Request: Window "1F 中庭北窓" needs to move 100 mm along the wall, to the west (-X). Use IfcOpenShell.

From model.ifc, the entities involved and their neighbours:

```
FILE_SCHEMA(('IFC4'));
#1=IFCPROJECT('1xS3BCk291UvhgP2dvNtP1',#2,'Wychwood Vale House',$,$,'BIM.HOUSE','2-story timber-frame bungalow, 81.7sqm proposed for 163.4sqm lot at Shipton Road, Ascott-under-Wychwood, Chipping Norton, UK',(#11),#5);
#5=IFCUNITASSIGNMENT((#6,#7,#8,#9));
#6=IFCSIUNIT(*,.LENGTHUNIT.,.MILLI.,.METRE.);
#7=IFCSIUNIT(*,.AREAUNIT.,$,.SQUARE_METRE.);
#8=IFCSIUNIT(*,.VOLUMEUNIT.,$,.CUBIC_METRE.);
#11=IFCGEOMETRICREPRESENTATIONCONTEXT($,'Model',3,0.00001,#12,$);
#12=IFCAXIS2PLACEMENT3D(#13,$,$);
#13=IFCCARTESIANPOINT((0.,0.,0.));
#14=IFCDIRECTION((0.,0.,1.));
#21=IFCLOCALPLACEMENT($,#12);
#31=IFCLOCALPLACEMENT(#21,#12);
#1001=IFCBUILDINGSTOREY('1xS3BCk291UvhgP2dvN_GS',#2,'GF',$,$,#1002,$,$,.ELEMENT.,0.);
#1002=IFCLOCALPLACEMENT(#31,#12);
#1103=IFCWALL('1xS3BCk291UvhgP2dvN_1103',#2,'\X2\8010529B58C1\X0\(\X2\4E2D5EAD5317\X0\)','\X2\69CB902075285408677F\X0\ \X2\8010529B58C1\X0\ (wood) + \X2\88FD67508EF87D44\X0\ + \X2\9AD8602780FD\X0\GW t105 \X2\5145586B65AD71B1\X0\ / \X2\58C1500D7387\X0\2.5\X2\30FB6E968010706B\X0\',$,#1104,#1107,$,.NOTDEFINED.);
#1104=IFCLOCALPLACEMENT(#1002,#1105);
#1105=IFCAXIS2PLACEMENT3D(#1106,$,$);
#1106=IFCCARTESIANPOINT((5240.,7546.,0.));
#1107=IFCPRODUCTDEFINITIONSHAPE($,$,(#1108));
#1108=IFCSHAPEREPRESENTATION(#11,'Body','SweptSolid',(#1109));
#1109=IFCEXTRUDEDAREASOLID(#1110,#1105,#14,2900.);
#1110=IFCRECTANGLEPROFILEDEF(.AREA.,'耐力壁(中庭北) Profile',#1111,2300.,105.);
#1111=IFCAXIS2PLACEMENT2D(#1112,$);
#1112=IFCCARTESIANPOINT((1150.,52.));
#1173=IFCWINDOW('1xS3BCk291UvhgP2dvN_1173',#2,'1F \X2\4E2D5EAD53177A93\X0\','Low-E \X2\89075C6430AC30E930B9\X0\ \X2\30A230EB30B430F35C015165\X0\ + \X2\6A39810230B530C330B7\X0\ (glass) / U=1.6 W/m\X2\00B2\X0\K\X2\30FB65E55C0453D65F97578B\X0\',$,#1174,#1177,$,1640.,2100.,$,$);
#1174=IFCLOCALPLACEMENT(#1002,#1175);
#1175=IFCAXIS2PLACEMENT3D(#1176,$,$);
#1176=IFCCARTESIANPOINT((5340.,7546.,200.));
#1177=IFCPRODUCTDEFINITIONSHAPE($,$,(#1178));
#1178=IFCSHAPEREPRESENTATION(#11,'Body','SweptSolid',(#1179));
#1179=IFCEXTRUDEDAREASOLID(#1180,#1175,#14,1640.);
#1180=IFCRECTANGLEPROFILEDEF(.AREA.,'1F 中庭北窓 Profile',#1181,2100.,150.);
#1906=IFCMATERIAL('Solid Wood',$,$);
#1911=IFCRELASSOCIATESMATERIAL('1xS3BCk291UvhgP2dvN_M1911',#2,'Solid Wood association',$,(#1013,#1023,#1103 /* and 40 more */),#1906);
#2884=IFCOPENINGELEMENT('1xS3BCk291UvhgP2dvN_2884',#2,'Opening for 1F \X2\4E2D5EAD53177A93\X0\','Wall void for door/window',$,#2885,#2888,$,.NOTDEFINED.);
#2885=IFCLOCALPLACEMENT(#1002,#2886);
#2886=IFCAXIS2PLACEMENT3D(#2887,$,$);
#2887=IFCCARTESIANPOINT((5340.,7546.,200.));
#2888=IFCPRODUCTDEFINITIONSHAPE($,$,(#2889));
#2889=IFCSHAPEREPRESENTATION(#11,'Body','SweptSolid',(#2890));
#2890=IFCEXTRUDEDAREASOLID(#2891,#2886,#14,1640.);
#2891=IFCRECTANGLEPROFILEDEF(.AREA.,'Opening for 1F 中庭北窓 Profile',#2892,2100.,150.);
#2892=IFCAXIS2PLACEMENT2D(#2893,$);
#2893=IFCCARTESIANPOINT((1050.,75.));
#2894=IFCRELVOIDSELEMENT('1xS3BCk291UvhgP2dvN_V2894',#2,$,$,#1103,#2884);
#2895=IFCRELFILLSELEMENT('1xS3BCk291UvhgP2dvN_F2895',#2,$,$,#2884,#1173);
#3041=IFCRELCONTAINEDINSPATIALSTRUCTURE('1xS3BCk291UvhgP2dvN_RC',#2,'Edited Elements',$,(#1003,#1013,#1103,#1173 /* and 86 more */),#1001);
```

```python
import ifcopenshell
import ifcopenshell.api.geometry
import ifcopenshell.util.placement
import ifcopenshell.util.unit

model = ifcopenshell.open("model.ifc")
unit_scale = ifcopenshell.util.unit.calculate_unit_scale(model)

window = model.by_id(1173)
opening = window.FillsVoids[0].RelatingOpeningElement
wall = opening.VoidsElements[0].RelatingBuildingElement

wall_matrix = ifcopenshell.util.placement.get_local_placement(wall.ObjectPlacement)
shift = wall_matrix[:3, 0] * -0.1 / unit_scale
before = ifcopenshell.util.placement.get_local_placement(window.ObjectPlacement)[:3, 3].copy()

# The window is not placed relative to its opening, so move both.
for product in (opening, window):
    matrix = ifcopenshell.util.placement.get_local_placement(product.ObjectPlacement)
    matrix[:3, 3] += shift
    ifcopenshell.api.geometry.edit_object_placement(model, product=product, matrix=matrix, is_si=False)

after = ifcopenshell.util.placement.get_local_placement(window.ObjectPlacement)[:3, 3]
print("window moved by", (after - before).round(3) + 0.0)

model.write("model_updated.ifc")
```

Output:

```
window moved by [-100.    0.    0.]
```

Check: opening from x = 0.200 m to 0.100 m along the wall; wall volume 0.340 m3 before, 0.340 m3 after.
